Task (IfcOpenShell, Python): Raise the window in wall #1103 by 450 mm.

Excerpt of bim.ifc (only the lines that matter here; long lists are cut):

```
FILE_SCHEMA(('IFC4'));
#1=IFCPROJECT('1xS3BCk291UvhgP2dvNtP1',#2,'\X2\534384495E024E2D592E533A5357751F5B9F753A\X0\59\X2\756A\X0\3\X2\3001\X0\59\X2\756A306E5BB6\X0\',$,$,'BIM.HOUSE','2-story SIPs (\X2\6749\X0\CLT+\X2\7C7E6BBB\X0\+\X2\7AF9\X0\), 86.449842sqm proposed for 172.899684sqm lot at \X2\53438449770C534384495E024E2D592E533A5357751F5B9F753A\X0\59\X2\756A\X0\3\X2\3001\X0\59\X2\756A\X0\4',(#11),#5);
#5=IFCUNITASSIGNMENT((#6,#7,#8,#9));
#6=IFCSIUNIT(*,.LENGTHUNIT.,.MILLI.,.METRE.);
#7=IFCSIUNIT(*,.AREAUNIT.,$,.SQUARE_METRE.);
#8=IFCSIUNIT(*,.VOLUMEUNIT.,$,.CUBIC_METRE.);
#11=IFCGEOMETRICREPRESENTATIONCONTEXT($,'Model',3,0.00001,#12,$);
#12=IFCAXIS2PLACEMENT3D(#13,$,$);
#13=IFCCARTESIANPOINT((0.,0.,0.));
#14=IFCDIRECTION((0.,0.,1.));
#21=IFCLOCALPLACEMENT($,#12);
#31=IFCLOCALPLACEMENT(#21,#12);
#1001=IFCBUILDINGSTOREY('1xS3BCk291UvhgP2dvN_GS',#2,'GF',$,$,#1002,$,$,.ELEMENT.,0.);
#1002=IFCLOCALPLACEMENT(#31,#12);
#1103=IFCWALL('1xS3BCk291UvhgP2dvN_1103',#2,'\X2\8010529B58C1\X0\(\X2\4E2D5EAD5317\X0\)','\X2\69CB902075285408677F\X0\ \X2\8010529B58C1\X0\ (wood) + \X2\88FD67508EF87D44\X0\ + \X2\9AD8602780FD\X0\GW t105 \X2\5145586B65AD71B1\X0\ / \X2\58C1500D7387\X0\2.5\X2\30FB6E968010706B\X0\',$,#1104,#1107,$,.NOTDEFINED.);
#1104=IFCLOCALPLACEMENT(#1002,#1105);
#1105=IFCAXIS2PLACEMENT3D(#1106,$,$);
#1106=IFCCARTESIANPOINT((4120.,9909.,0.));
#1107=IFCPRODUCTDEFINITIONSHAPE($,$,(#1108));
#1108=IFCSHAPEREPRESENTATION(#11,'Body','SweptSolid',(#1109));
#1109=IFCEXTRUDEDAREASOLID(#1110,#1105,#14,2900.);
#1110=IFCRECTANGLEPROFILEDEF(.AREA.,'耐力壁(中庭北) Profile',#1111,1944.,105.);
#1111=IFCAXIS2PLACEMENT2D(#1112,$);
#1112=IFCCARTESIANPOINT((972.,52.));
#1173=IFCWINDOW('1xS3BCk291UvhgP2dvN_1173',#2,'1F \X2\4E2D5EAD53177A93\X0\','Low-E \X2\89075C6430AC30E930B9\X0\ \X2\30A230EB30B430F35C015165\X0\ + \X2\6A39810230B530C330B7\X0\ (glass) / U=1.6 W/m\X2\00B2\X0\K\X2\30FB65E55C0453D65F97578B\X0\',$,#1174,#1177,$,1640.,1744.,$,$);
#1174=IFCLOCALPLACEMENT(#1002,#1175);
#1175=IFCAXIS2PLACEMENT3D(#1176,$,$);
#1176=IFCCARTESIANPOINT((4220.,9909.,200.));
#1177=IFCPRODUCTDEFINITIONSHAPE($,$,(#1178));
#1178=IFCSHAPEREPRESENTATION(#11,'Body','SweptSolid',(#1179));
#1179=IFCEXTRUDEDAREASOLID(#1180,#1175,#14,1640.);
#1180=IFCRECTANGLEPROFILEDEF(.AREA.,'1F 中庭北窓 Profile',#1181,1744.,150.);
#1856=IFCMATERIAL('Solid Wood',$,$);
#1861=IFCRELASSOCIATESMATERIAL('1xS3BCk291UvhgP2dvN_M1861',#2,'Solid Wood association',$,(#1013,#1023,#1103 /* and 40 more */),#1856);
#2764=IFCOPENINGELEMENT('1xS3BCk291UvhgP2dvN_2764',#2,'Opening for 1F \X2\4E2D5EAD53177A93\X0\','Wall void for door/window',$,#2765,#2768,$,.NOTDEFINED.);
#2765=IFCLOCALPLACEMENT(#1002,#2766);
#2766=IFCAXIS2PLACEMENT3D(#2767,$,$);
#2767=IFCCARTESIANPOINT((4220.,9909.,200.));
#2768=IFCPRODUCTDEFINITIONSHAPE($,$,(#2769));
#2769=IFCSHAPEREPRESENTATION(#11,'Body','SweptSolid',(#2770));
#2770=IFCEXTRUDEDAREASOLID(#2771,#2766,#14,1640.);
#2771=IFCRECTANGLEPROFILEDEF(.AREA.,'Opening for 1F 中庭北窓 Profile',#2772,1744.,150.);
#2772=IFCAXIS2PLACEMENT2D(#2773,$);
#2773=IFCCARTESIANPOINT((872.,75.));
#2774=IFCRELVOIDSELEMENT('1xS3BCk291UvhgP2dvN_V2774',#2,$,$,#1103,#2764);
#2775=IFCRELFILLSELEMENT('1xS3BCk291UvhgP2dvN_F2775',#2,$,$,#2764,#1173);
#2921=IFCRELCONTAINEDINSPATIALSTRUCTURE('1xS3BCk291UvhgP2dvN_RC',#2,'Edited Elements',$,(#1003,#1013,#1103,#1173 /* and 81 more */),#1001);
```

```python
import numpy as np
import ifcopenshell
import ifcopenshell.api.geometry
import ifcopenshell.util.placement
import ifcopenshell.util.unit

model = ifcopenshell.open("bim.ifc")
unit_scale = ifcopenshell.util.unit.calculate_unit_scale(model)

window = model.by_guid("1xS3BCk291UvhgP2dvN_1173")
opening = window.FillsVoids[0].RelatingOpeningElement
dz = 0.45 / unit_scale

shift = np.array([0.0, 0.0, dz])
# The window is not placed relative to its opening, so move both.
for product in (opening, window):
    matrix = ifcopenshell.util.placement.get_local_placement(product.ObjectPlacement)
    matrix[:3, 3] += shift
    ifcopenshell.api.geometry.edit_object_placement(model, product=product, matrix=matrix, is_si=False)

print(f"moved by {dz * unit_scale:+.3f} m")

model.write("bim_updated.ifc")
```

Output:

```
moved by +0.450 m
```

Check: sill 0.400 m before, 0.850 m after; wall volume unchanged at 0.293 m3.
